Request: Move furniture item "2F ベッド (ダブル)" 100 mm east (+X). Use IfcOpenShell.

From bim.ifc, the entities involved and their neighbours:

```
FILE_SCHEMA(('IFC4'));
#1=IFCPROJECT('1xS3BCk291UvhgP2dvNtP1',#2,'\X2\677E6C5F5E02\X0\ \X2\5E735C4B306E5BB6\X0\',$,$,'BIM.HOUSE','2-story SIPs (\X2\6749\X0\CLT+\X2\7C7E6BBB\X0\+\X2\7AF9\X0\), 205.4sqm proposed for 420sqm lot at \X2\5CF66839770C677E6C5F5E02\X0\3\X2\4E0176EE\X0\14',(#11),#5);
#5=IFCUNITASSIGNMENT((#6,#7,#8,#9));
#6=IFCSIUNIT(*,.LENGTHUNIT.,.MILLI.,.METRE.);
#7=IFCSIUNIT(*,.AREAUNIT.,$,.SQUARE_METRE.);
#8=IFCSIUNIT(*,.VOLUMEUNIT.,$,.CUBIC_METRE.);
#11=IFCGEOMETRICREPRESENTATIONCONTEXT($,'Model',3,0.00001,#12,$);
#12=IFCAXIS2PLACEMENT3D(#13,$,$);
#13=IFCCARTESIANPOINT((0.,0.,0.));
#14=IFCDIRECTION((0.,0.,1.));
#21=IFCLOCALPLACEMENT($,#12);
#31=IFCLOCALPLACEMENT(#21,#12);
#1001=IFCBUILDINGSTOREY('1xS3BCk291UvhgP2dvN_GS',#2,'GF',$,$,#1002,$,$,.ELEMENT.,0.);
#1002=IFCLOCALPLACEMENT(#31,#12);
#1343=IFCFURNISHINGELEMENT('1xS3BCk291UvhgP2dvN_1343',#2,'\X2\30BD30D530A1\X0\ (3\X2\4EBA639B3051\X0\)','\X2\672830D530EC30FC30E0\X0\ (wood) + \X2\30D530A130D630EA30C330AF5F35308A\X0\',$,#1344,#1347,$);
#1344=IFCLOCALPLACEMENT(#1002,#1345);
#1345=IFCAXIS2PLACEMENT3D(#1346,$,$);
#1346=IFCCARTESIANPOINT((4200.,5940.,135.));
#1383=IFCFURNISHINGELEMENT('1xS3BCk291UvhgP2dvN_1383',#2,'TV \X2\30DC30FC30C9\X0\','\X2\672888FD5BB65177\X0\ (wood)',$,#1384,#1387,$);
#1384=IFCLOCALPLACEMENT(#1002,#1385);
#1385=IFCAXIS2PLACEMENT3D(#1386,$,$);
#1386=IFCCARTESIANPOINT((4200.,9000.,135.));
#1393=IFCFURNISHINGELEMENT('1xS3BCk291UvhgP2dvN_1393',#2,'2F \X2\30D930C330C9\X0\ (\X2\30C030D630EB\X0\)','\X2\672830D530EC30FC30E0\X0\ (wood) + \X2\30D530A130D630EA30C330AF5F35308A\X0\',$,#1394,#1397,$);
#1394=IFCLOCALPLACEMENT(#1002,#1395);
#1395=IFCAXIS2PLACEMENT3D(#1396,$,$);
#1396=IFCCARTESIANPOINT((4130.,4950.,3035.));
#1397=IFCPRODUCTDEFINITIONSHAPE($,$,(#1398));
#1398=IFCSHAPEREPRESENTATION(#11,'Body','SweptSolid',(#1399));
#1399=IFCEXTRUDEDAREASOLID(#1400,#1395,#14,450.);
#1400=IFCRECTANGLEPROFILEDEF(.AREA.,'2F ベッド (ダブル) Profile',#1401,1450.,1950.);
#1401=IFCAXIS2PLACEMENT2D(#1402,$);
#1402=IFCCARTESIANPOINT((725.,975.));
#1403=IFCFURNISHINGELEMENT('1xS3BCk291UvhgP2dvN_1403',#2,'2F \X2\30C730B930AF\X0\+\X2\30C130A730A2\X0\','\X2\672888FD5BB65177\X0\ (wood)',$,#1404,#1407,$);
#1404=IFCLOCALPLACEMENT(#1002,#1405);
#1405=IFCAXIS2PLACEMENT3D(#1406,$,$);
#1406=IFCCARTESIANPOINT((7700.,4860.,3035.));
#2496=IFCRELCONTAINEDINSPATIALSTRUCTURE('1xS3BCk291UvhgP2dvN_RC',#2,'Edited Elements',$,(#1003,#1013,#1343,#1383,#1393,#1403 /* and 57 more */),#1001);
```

```python
import ifcopenshell
import ifcopenshell.api.geometry
import ifcopenshell.util.placement

model = ifcopenshell.open("bim.ifc")

item = model.by_guid("1xS3BCk291UvhgP2dvN_1393")
matrix = ifcopenshell.util.placement.get_local_placement(item.ObjectPlacement)
matrix[0, 3] += 100.0
ifcopenshell.api.geometry.edit_object_placement(model, product=item, matrix=matrix, is_si=False)

print(ifcopenshell.util.placement.get_local_placement(item.ObjectPlacement).round(3) + 0.0)

model.write("bim_edited.ifc")
```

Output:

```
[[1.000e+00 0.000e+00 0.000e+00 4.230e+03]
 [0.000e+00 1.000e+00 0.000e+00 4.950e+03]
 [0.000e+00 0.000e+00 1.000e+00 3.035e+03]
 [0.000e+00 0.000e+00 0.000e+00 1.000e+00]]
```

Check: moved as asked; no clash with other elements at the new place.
